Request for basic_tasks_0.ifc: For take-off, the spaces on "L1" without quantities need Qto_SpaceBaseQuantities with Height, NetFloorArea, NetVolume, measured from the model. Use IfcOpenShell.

First a look at what the model holds.

```python
import ifcopenshell
import ifcopenshell.util.element
import ifcopenshell.util.unit

model = ifcopenshell.open("basic_tasks_0.ifc")
print(model.schema)
for unit_type in ("LENGTHUNIT", "AREAUNIT", "VOLUMEUNIT"):
    print(unit_type, ifcopenshell.util.unit.calculate_unit_scale(model, unit_type))
storey = next(s for s in model.by_type("IfcBuildingStorey") if s.Name == "L1")
spaces = [e for e in ifcopenshell.util.element.get_decomposition(storey) if e.is_a("IfcSpace")]
for e in sorted(spaces, key=lambda e: e.id()):
    print(e.id(), e.is_a(), e.Name, list(ifcopenshell.util.element.get_psets(e, qtos_only=True)), sep=" | ")
```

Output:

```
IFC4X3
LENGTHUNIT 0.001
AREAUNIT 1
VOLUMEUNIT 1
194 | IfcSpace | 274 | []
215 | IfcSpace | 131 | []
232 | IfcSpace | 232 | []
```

```python
import ifcopenshell
import ifcopenshell.api.pset
import ifcopenshell.geom
import ifcopenshell.util.element
import ifcopenshell.util.shape
import ifcopenshell.util.unit

model = ifcopenshell.open("basic_tasks_0.ifc")
unit_scale = ifcopenshell.util.unit.calculate_unit_scale(model)
area_scale = ifcopenshell.util.unit.calculate_unit_scale(model, "AREAUNIT")
volume_scale = ifcopenshell.util.unit.calculate_unit_scale(model, "VOLUMEUNIT")
settings = ifcopenshell.geom.settings()

storey = next(s for s in model.by_type("IfcBuildingStorey") if s.Name == "L1")
spaces = [e for e in ifcopenshell.util.element.get_decomposition(storey) if e.is_a("IfcSpace")]

for e in sorted(spaces, key=lambda e: e.id()):
    if ifcopenshell.util.element.get_psets(e, qtos_only=True, should_inherit=False):
        continue
    # Geometry comes back in metres, in the element's own axes.
    shape = ifcopenshell.geom.create_shape(settings, e)
    values = {
        "Height": ifcopenshell.util.shape.get_z(shape.geometry) / unit_scale,
        "NetFloorArea": ifcopenshell.util.shape.get_footprint_area(shape.geometry) / area_scale,
        "NetVolume": ifcopenshell.util.shape.get_volume(shape.geometry) / volume_scale,
    }
    qto = ifcopenshell.api.pset.add_qto(model, product=e, name="Qto_SpaceBaseQuantities")
    ifcopenshell.api.pset.edit_qto(model, qto=qto, properties=values)
    print(e.id(), {k: round(v, 3) for k, v in values.items()})

model.write("basic_tasks_0_rev.ifc")
```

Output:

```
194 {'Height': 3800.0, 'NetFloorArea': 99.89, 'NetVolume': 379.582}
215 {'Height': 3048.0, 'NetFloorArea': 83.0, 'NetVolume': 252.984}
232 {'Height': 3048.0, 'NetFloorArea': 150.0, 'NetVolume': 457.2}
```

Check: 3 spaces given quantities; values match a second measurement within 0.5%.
